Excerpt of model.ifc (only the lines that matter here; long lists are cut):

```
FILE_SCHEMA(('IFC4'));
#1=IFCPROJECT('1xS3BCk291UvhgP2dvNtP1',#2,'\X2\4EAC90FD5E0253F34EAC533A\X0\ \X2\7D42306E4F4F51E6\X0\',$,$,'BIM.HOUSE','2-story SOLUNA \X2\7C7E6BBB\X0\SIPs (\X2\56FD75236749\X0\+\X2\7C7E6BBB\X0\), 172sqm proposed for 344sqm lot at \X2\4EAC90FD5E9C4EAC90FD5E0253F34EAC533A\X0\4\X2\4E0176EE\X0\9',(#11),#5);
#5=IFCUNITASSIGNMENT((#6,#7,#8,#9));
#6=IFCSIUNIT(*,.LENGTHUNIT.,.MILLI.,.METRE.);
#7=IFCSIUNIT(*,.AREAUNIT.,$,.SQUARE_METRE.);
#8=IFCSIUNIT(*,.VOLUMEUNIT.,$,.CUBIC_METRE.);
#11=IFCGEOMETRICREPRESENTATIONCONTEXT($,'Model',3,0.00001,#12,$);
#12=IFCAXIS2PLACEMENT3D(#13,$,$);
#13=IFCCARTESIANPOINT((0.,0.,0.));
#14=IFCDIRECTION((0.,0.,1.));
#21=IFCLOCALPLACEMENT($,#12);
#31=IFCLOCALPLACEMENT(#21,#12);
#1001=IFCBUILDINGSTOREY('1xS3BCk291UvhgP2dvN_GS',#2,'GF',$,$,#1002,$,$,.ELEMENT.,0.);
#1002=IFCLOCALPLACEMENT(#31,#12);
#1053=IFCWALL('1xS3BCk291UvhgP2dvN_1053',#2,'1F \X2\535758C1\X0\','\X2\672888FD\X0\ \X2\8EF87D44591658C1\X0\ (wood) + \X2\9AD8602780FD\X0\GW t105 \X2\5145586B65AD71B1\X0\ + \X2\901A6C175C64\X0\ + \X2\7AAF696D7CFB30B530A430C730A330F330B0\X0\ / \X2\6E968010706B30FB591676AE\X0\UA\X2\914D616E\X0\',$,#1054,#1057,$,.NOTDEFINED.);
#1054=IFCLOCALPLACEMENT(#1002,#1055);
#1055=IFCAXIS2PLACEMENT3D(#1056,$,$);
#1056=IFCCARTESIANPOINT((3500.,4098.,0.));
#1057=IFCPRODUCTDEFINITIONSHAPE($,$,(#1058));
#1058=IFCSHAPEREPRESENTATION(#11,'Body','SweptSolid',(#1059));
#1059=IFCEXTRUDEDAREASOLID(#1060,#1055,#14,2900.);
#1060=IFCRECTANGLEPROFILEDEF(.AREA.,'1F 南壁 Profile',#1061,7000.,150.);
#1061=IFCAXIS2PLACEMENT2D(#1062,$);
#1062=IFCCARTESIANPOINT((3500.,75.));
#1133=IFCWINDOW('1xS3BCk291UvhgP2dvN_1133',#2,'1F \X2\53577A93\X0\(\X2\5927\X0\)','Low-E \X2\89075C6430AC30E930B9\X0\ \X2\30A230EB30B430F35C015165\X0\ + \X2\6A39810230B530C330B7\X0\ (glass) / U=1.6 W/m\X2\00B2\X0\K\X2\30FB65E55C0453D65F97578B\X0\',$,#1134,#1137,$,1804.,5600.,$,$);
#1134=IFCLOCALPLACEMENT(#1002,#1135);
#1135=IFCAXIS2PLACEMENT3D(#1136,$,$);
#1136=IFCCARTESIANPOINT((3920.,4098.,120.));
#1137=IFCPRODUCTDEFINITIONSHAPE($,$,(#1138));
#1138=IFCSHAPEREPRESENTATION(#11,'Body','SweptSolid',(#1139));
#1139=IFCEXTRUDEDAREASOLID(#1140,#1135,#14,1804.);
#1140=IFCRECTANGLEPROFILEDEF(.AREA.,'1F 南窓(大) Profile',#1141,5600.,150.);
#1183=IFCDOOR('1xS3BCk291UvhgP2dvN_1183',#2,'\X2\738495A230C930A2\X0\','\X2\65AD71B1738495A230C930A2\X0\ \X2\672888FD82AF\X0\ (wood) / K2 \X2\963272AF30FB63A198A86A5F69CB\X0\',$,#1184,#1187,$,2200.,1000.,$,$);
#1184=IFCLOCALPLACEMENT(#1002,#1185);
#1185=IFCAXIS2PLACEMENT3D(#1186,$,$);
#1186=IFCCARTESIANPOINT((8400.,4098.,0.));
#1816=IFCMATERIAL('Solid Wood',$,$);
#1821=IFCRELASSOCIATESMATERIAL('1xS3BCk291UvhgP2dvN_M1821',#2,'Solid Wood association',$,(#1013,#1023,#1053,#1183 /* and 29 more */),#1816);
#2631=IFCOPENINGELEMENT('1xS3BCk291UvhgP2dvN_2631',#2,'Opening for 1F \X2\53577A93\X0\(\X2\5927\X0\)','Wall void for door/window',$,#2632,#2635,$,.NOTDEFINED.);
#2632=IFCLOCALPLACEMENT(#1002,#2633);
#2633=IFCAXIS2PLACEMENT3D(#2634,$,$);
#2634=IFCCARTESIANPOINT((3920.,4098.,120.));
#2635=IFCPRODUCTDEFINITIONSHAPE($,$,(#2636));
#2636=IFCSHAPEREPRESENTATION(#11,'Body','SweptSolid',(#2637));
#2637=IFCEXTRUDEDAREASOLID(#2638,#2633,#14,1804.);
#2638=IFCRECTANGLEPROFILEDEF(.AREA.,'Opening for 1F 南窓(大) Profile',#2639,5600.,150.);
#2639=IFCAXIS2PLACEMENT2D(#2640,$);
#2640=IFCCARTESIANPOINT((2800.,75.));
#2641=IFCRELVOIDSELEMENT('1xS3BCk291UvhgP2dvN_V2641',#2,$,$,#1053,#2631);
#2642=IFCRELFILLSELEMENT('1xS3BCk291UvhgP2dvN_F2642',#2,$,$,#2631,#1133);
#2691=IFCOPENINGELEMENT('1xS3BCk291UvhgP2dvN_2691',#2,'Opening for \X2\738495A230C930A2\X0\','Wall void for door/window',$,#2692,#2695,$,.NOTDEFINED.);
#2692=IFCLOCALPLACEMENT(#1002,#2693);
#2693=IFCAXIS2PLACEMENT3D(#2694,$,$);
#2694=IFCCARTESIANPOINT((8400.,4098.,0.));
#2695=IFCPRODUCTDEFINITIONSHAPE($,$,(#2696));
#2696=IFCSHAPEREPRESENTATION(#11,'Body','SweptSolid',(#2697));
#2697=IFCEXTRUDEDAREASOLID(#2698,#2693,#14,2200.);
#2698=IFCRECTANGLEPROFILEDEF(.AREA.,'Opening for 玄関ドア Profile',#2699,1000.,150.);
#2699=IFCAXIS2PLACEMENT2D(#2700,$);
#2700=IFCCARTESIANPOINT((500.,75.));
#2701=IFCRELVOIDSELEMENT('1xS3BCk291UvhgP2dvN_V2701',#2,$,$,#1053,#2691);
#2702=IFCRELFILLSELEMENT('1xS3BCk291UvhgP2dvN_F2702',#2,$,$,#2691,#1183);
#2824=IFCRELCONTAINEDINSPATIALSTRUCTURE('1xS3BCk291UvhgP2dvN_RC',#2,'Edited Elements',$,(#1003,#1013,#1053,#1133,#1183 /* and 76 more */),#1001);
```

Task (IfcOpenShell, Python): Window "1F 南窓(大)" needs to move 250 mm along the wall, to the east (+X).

```python
import ifcopenshell
import ifcopenshell.api.geometry
import ifcopenshell.util.placement
import ifcopenshell.util.unit

model = ifcopenshell.open("model.ifc")
unit_scale = ifcopenshell.util.unit.calculate_unit_scale(model)

window = model.by_guid("1xS3BCk291UvhgP2dvN_1133")
opening = window.FillsVoids[0].RelatingOpeningElement
wall = opening.VoidsElements[0].RelatingBuildingElement

wall_matrix = ifcopenshell.util.placement.get_local_placement(wall.ObjectPlacement)
shift = wall_matrix[:3, 0] * 0.25 / unit_scale
before = ifcopenshell.util.placement.get_local_placement(window.ObjectPlacement)[:3, 3].copy()

# The window is not placed relative to its opening, so move both.
for product in (opening, window):
    matrix = ifcopenshell.util.placement.get_local_placement(product.ObjectPlacement)
    matrix[:3, 3] += shift
    ifcopenshell.api.geometry.edit_object_placement(model, product=product, matrix=matrix, is_si=False)

after = ifcopenshell.util.placement.get_local_placement(window.ObjectPlacement)[:3, 3]
print("window moved by", (after - before).round(3) + 0.0)

model.write("model_v2.ifc")
```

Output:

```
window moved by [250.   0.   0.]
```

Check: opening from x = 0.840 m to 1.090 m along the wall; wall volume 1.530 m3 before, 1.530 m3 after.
